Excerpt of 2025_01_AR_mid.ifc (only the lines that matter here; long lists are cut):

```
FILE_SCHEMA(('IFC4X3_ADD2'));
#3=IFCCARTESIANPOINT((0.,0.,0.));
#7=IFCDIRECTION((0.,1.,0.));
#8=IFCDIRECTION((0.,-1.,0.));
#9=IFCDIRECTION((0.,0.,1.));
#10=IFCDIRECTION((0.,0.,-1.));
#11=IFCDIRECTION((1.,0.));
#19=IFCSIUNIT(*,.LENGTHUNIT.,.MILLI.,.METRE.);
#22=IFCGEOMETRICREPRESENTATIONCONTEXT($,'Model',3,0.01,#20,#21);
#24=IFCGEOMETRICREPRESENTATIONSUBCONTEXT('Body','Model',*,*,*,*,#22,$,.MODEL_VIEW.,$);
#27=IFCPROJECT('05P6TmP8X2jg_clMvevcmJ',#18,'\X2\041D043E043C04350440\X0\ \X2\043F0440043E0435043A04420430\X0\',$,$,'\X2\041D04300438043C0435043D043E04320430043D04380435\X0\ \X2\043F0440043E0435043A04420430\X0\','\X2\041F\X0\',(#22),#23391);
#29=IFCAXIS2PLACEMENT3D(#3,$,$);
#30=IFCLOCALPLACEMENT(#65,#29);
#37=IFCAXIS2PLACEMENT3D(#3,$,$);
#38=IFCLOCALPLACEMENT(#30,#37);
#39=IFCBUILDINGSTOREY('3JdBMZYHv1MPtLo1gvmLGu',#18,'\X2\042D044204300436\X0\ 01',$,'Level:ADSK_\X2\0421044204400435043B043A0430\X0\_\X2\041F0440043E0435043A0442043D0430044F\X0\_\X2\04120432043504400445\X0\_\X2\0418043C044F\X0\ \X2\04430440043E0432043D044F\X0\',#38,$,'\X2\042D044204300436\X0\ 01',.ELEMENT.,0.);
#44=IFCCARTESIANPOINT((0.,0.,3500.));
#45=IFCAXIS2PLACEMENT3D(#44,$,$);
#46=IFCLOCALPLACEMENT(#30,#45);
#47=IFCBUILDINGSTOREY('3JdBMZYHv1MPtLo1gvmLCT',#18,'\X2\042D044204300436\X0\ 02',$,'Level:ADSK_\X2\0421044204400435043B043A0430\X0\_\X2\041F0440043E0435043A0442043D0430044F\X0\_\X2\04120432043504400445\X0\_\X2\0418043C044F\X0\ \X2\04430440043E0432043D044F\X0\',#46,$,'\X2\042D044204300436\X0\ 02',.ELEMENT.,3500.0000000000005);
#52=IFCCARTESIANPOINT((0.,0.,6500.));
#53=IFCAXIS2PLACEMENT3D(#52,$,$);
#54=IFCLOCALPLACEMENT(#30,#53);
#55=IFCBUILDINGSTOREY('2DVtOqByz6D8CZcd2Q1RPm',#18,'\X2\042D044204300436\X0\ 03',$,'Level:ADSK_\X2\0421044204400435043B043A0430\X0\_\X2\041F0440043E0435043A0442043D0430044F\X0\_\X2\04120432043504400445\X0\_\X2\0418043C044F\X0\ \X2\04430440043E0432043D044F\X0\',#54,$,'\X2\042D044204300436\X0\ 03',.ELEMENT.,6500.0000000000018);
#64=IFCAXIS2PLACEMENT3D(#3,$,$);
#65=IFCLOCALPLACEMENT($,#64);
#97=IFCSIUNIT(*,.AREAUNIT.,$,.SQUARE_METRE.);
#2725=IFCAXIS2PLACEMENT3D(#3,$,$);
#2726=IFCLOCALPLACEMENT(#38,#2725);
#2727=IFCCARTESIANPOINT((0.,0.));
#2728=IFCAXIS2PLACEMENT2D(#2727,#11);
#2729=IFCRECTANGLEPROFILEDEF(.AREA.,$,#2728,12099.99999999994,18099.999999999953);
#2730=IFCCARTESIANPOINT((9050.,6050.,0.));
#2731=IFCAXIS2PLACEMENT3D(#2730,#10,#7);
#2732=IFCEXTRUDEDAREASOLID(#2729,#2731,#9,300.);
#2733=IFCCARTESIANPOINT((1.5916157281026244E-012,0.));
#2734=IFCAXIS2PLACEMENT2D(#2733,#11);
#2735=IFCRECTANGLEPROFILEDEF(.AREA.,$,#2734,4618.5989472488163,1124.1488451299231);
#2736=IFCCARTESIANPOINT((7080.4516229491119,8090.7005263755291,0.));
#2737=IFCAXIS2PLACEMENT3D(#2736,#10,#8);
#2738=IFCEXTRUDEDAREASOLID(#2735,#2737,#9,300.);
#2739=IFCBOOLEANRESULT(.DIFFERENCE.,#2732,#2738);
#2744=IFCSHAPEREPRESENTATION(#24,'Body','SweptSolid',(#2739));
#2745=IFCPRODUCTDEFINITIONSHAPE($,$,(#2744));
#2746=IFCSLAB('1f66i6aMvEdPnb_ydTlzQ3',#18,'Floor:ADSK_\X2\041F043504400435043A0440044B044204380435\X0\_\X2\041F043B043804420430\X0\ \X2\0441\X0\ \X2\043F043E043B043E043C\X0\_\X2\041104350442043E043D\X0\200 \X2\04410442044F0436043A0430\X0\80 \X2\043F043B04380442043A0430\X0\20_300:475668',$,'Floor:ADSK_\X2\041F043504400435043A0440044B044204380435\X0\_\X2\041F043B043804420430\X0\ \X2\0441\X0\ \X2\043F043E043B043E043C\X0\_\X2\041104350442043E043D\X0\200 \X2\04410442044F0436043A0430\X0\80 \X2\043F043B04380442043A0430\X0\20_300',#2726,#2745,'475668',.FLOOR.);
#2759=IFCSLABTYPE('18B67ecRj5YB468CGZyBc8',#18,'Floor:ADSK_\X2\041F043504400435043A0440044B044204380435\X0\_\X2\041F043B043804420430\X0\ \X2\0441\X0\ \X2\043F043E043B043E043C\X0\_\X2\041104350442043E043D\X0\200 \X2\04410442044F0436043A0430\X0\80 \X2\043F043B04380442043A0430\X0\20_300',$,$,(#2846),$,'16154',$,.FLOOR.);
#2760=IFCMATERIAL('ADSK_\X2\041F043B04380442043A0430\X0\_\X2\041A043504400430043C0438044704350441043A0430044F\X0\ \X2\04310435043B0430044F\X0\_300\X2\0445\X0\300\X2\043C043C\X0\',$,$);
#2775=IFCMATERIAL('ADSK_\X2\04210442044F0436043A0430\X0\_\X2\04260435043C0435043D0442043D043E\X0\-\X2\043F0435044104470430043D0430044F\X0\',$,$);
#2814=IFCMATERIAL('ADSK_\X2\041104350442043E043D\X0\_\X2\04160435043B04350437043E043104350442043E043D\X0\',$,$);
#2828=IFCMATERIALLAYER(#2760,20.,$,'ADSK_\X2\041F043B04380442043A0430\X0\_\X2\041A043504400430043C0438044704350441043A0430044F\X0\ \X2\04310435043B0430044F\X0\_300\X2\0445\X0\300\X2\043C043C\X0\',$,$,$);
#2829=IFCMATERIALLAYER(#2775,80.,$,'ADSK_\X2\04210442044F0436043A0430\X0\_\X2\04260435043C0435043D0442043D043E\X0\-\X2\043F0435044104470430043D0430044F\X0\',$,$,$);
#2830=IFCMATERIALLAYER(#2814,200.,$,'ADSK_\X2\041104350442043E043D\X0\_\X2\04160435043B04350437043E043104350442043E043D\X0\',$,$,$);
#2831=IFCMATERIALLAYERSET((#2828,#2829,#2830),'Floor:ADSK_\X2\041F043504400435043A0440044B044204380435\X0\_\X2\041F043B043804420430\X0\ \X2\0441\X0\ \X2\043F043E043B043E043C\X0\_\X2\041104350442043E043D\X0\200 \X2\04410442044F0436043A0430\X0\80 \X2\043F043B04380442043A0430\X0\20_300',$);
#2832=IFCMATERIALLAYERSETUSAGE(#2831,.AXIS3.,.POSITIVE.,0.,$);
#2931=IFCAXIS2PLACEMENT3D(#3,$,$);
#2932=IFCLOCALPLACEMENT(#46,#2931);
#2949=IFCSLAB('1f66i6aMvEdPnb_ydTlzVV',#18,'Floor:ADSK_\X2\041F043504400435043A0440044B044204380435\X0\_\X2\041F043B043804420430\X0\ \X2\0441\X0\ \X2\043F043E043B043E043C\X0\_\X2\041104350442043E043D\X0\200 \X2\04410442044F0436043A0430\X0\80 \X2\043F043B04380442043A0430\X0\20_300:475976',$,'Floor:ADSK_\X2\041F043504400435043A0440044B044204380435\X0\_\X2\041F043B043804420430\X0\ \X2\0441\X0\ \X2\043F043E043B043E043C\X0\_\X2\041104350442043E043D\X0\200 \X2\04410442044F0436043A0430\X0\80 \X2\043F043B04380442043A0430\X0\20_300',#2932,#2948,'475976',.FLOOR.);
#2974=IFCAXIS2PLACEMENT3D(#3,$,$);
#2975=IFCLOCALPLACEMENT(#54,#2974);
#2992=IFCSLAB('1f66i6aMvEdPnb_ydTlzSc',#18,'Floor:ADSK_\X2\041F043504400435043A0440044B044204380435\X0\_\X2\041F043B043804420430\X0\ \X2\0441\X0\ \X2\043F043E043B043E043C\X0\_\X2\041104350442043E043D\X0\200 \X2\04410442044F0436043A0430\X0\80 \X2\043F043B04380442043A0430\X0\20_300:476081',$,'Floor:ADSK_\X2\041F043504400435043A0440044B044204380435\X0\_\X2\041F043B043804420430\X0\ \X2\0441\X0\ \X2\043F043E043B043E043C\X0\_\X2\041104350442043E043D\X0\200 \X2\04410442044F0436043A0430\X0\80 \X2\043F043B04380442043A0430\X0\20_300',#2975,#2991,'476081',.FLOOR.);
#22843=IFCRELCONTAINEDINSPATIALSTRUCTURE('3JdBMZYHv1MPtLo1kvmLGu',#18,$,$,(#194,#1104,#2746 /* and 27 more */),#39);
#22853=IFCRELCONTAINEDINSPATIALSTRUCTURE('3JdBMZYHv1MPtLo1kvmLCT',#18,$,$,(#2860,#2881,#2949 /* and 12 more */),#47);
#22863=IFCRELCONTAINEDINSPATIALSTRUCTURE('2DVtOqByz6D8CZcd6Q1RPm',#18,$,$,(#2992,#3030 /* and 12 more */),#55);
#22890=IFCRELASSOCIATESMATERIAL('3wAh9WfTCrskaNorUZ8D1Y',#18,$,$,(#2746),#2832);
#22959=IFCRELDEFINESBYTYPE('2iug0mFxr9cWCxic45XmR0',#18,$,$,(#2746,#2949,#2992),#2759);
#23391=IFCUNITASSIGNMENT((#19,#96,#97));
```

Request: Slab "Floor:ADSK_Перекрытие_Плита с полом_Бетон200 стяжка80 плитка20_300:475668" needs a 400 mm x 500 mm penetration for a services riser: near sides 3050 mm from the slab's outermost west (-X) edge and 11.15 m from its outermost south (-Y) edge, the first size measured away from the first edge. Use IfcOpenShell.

```python
import numpy as np
import ifcopenshell
import ifcopenshell.api.feature
import ifcopenshell.api.geometry
import ifcopenshell.api.root
import ifcopenshell.geom
import ifcopenshell.util.placement
import ifcopenshell.util.representation
import ifcopenshell.util.shape
import ifcopenshell.util.unit

model = ifcopenshell.open("2025_01_AR_mid.ifc")
unit_scale = ifcopenshell.util.unit.calculate_unit_scale(model)
settings = ifcopenshell.geom.settings()


def volume(element):
    """Net volume in cubic metres, openings subtracted."""
    shape = ifcopenshell.geom.create_shape(settings, element)
    return ifcopenshell.util.shape.get_volume(shape.geometry)


slab = model.by_guid("1f66i6aMvEdPnb_ydTlzQ3")
before = volume(slab)

# Extent in the slab's own axes, in metres. The edges named are its -X and -Y sides.
slab_shape = ifcopenshell.geom.create_shape(settings, slab)
vertices = ifcopenshell.util.shape.get_vertices(slab_shape.geometry)
x_min, y_min, bottom = vertices.min(axis=0)
top = vertices[:, 2].max()

opening = ifcopenshell.api.root.create_entity(model, ifc_class="IfcOpeningElement", name="Services riser opening", predefined_type="OPENING")
context = ifcopenshell.util.representation.get_context(model, "Model", "Body", "MODEL_VIEW")
width, depth = 0.4, 0.5
outline = [(0.0, 0.0), (width, 0.0), (width, depth), (0.0, depth), (0.0, 0.0)]
# Overshoot both faces by 50 mm so the cut is clean.
shape = ifcopenshell.api.geometry.add_slab_representation(
    model, context=context, depth=top - bottom + 0.1, polyline=outline
)
ifcopenshell.api.geometry.assign_representation(model, product=opening, representation=shape)

matrix = ifcopenshell.util.placement.get_local_placement(slab.ObjectPlacement)
matrix[:, 3] = matrix @ np.append(np.array([x_min + 3.05, y_min + 11.15, bottom - 0.05]) / unit_scale, 1.0)
ifcopenshell.api.geometry.edit_object_placement(model, product=opening, matrix=matrix, is_si=False)
ifcopenshell.api.feature.add_feature(model, feature=opening, element=slab)

after = volume(slab)

print(f"slab volume {before:.3f} -> {after:.3f} m3")

model.write("2025_01_AR_mid_edited.ifc")
```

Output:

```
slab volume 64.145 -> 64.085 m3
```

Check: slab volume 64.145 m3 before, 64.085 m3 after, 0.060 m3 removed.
